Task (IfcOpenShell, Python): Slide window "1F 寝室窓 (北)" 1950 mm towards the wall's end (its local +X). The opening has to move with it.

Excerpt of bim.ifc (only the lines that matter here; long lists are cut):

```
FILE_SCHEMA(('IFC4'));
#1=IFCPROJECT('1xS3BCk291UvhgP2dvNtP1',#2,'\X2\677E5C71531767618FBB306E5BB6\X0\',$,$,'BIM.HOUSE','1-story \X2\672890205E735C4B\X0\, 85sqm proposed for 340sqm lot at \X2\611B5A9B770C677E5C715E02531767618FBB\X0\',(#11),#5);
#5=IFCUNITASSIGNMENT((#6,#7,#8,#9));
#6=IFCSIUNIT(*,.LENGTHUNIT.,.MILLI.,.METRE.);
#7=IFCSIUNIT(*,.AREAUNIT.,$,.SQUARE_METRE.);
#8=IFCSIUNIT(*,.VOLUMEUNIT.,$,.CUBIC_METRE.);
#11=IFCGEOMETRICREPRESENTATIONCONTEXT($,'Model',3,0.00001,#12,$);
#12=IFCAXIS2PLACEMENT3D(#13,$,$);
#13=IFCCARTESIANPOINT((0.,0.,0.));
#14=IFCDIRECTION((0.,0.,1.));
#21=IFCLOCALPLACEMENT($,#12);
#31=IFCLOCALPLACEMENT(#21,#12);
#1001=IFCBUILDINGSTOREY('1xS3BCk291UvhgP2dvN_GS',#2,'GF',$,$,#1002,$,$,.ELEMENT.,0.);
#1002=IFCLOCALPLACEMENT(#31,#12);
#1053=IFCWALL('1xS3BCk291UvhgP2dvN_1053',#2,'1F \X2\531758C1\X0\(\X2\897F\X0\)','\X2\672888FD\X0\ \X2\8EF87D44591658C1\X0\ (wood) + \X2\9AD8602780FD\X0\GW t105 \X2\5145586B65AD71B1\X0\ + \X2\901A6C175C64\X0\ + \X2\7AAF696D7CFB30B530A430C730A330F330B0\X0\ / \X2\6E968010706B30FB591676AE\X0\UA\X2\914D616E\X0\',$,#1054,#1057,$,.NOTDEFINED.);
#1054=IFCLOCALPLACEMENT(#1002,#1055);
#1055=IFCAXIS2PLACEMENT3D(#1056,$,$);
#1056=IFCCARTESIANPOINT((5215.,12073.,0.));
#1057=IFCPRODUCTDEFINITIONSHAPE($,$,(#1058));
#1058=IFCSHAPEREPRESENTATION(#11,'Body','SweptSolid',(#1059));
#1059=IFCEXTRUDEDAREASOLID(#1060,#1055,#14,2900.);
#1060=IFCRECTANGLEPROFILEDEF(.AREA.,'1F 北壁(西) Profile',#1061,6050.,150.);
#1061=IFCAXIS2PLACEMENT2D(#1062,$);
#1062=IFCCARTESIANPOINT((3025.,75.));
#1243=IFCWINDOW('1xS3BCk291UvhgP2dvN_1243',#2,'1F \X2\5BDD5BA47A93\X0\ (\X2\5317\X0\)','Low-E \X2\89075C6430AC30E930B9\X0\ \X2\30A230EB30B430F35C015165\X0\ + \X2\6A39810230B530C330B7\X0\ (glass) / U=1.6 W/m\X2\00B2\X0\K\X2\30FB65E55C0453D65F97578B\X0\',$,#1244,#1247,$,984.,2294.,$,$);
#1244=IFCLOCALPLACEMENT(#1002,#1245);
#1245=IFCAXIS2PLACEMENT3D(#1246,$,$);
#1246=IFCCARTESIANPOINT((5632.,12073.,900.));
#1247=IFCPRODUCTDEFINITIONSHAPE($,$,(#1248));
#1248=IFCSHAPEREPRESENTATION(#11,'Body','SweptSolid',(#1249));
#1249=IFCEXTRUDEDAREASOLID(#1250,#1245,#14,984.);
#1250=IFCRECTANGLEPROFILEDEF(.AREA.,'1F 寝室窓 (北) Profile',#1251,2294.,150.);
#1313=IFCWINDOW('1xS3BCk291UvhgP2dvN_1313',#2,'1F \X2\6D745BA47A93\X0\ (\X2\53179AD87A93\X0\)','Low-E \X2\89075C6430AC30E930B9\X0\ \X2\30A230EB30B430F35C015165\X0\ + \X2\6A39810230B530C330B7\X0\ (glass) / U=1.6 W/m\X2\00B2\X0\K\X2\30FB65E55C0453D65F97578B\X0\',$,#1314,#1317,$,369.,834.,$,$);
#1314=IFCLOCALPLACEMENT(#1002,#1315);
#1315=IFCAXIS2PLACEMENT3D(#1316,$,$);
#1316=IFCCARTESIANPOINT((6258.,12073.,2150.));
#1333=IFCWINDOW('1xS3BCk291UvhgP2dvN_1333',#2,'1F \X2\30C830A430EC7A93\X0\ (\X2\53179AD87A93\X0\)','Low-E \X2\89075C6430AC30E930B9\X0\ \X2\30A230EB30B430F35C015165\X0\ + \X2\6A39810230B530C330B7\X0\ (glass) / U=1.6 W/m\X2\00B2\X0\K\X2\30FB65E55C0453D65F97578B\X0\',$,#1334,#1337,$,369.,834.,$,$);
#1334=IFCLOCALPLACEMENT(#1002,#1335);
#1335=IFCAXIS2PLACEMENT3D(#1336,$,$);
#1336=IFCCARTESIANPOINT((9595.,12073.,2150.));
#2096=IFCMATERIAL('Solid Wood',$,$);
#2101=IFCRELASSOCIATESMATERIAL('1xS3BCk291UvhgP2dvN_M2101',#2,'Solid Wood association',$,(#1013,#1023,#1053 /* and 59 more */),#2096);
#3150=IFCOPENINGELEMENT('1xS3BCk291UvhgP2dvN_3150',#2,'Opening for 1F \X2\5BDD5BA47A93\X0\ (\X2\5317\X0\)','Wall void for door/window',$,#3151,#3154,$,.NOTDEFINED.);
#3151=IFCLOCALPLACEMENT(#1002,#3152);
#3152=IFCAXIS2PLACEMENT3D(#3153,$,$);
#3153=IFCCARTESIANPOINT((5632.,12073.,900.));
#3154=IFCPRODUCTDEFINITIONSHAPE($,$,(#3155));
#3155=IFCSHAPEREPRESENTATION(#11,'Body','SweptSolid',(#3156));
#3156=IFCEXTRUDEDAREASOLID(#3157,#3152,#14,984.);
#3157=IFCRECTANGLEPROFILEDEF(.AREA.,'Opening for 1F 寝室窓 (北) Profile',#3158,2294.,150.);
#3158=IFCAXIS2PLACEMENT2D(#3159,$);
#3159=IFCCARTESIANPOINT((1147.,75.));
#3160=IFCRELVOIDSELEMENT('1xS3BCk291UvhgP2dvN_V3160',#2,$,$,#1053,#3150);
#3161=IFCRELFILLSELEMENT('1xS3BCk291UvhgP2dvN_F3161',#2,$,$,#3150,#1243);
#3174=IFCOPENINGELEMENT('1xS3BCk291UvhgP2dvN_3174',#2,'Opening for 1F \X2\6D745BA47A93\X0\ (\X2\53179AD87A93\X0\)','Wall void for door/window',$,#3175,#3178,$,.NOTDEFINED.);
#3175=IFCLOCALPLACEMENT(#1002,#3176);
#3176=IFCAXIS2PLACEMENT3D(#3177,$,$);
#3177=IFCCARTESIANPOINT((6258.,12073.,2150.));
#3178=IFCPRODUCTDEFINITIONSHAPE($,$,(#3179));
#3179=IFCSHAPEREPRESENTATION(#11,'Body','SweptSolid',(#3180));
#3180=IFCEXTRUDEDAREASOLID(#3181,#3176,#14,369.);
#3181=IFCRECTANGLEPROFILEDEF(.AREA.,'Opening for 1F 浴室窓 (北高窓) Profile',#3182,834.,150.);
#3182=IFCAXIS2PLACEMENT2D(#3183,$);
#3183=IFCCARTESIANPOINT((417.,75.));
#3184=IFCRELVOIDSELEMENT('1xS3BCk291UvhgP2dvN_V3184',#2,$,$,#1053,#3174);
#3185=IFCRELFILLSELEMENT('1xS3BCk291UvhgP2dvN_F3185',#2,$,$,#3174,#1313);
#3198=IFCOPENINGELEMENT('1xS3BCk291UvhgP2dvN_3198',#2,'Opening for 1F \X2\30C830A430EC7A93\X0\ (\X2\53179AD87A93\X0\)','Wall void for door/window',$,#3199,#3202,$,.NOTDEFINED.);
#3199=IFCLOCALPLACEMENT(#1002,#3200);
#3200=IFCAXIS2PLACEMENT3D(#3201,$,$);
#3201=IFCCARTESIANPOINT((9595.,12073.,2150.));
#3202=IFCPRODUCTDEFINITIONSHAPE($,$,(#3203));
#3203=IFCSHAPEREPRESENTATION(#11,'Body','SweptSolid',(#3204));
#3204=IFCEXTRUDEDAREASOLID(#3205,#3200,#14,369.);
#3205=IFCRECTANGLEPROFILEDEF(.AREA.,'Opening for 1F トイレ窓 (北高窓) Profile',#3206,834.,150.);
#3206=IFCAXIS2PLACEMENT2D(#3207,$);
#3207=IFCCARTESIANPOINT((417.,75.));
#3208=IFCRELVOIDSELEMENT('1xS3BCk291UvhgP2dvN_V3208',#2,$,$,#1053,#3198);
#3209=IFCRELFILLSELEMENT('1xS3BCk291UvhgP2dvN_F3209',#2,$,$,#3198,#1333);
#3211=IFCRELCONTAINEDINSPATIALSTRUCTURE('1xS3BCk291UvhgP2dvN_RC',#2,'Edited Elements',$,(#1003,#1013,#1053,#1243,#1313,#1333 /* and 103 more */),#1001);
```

```python
import ifcopenshell
import ifcopenshell.api.geometry
import ifcopenshell.util.placement
import ifcopenshell.util.unit

model = ifcopenshell.open("bim.ifc")
unit_scale = ifcopenshell.util.unit.calculate_unit_scale(model)

window = model.by_guid("1xS3BCk291UvhgP2dvN_1243")
opening = window.FillsVoids[0].RelatingOpeningElement
wall = opening.VoidsElements[0].RelatingBuildingElement

wall_matrix = ifcopenshell.util.placement.get_local_placement(wall.ObjectPlacement)
shift = wall_matrix[:3, 0] * 1.95 / unit_scale
before = ifcopenshell.util.placement.get_local_placement(window.ObjectPlacement)[:3, 3].copy()

# The window is not placed relative to its opening, so move both.
for product in (opening, window):
    matrix = ifcopenshell.util.placement.get_local_placement(product.ObjectPlacement)
    matrix[:3, 3] += shift
    ifcopenshell.api.geometry.edit_object_placement(model, product=product, matrix=matrix, is_si=False)

after = ifcopenshell.util.placement.get_local_placement(window.ObjectPlacement)[:3, 3]
print("window moved by", (after - before).round(3) + 0.0)

model.write("bim_v2.ifc")
```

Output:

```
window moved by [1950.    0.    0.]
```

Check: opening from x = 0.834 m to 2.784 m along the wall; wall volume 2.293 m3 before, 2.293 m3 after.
